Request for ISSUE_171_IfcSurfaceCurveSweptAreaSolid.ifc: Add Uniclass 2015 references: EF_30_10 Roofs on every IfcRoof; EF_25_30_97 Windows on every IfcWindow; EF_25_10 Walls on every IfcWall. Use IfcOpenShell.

First a look at what the model holds.

```python
import ifcopenshell

model = ifcopenshell.open("ISSUE_171_IfcSurfaceCurveSweptAreaSolid.ifc")
print(model.schema)
print("classifications:", [c.Name for c in model.by_type("IfcClassification")])
for ifc_class in ("IfcDoor", "IfcRoof", "IfcStair", "IfcWall", "IfcWindow"):
    print(ifc_class, len(model.by_type(ifc_class)))
```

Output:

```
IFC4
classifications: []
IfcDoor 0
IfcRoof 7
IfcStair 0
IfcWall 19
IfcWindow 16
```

```python
import ifcopenshell
import ifcopenshell.api.classification

model = ifcopenshell.open("ISSUE_171_IfcSurfaceCurveSweptAreaSolid.ifc")

system = ifcopenshell.api.classification.add_classification(model, classification="Uniclass 2015")

codes = {
    "IfcRoof": ("EF_30_10", "Roofs"),
    "IfcWindow": ("EF_25_30_97", "Windows"),
    "IfcWall": ("EF_25_10", "Walls"),
}
for ifc_class, (code, name) in codes.items():
    products = model.by_type(ifc_class)
    ifcopenshell.api.classification.add_reference(
        model, products=products, classification=system, identification=code, name=name
    )
    print(code, len(products))

model.write("ISSUE_171_IfcSurfaceCurveSweptAreaSolid_updated.ifc")
```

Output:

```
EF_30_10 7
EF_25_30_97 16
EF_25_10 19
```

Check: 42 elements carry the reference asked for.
